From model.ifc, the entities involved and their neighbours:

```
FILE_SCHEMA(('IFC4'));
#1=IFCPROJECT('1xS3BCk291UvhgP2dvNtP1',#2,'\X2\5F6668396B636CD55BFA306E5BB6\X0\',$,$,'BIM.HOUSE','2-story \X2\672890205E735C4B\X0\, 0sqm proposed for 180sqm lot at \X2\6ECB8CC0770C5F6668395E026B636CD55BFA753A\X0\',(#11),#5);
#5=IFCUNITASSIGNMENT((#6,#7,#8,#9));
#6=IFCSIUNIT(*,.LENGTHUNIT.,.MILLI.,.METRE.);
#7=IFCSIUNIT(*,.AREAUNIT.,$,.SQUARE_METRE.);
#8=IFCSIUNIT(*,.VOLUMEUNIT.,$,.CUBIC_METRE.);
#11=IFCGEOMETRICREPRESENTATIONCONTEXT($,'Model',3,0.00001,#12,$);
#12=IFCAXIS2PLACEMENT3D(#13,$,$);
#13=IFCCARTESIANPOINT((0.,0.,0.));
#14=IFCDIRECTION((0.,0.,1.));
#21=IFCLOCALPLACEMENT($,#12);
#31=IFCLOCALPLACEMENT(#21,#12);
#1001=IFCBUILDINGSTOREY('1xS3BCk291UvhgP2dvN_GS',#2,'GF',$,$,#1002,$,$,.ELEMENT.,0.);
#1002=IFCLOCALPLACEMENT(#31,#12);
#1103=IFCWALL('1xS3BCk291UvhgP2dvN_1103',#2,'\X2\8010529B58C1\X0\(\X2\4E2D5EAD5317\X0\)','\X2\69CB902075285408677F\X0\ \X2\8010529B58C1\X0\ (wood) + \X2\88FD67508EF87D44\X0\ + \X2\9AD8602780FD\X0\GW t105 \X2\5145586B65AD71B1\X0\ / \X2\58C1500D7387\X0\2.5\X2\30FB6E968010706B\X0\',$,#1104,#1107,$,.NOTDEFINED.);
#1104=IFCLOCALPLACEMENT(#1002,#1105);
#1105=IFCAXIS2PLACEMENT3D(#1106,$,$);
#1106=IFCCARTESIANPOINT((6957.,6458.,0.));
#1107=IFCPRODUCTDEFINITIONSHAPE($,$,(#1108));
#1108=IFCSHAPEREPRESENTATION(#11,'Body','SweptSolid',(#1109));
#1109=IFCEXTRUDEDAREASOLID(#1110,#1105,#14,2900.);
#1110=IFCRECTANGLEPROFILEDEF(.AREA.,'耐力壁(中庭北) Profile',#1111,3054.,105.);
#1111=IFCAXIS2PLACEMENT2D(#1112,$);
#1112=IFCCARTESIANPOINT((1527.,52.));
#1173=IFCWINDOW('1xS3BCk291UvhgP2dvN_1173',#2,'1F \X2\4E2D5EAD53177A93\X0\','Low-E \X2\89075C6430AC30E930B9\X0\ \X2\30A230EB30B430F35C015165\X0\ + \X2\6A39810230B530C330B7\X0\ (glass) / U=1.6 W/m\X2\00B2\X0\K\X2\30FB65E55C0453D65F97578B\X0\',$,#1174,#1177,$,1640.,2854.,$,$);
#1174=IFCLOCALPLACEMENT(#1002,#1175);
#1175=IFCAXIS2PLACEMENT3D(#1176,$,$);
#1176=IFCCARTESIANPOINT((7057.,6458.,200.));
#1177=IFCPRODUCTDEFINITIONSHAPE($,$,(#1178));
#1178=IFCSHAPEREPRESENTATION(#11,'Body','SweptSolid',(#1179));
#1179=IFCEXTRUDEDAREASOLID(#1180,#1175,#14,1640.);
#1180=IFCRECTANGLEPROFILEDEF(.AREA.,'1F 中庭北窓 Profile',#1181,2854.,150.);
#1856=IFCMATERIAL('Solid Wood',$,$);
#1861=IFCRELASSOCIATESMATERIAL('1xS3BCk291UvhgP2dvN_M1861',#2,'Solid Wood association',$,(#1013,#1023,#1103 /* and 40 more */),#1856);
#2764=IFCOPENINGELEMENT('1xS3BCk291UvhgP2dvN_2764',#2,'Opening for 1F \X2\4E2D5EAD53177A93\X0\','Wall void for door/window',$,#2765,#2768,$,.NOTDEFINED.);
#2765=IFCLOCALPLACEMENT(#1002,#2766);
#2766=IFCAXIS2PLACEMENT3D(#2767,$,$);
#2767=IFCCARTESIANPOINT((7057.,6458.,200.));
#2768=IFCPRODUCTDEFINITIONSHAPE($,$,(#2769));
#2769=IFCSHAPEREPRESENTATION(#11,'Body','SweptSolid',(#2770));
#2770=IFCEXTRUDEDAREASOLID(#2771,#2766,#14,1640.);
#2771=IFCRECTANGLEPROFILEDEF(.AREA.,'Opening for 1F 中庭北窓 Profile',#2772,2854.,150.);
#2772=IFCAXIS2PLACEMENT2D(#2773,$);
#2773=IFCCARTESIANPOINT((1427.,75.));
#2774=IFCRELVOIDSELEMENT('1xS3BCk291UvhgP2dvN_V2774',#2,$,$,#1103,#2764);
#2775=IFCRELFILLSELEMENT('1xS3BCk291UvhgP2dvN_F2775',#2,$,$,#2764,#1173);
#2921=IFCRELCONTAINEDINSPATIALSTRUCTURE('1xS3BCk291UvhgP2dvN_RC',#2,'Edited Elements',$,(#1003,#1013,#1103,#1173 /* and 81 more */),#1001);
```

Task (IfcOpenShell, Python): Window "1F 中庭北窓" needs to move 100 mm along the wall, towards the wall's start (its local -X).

```python
import ifcopenshell
import ifcopenshell.api.geometry
import ifcopenshell.util.placement
import ifcopenshell.util.unit

model = ifcopenshell.open("model.ifc")
unit_scale = ifcopenshell.util.unit.calculate_unit_scale(model)

window = model.by_guid("1xS3BCk291UvhgP2dvN_1173")
opening = window.FillsVoids[0].RelatingOpeningElement
wall = opening.VoidsElements[0].RelatingBuildingElement

wall_matrix = ifcopenshell.util.placement.get_local_placement(wall.ObjectPlacement)
shift = wall_matrix[:3, 0] * -0.1 / unit_scale
before = ifcopenshell.util.placement.get_local_placement(window.ObjectPlacement)[:3, 3].copy()

# The window is not placed relative to its opening, so move both.
for product in (opening, window):
    matrix = ifcopenshell.util.placement.get_local_placement(product.ObjectPlacement)
    matrix[:3, 3] += shift
    ifcopenshell.api.geometry.edit_object_placement(model, product=product, matrix=matrix, is_si=False)

after = ifcopenshell.util.placement.get_local_placement(window.ObjectPlacement)[:3, 3]
print("window moved by", (after - before).round(3) + 0.0)

model.write("model_updated.ifc")
```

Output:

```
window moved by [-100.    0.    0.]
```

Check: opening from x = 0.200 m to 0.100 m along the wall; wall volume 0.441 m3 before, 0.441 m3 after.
